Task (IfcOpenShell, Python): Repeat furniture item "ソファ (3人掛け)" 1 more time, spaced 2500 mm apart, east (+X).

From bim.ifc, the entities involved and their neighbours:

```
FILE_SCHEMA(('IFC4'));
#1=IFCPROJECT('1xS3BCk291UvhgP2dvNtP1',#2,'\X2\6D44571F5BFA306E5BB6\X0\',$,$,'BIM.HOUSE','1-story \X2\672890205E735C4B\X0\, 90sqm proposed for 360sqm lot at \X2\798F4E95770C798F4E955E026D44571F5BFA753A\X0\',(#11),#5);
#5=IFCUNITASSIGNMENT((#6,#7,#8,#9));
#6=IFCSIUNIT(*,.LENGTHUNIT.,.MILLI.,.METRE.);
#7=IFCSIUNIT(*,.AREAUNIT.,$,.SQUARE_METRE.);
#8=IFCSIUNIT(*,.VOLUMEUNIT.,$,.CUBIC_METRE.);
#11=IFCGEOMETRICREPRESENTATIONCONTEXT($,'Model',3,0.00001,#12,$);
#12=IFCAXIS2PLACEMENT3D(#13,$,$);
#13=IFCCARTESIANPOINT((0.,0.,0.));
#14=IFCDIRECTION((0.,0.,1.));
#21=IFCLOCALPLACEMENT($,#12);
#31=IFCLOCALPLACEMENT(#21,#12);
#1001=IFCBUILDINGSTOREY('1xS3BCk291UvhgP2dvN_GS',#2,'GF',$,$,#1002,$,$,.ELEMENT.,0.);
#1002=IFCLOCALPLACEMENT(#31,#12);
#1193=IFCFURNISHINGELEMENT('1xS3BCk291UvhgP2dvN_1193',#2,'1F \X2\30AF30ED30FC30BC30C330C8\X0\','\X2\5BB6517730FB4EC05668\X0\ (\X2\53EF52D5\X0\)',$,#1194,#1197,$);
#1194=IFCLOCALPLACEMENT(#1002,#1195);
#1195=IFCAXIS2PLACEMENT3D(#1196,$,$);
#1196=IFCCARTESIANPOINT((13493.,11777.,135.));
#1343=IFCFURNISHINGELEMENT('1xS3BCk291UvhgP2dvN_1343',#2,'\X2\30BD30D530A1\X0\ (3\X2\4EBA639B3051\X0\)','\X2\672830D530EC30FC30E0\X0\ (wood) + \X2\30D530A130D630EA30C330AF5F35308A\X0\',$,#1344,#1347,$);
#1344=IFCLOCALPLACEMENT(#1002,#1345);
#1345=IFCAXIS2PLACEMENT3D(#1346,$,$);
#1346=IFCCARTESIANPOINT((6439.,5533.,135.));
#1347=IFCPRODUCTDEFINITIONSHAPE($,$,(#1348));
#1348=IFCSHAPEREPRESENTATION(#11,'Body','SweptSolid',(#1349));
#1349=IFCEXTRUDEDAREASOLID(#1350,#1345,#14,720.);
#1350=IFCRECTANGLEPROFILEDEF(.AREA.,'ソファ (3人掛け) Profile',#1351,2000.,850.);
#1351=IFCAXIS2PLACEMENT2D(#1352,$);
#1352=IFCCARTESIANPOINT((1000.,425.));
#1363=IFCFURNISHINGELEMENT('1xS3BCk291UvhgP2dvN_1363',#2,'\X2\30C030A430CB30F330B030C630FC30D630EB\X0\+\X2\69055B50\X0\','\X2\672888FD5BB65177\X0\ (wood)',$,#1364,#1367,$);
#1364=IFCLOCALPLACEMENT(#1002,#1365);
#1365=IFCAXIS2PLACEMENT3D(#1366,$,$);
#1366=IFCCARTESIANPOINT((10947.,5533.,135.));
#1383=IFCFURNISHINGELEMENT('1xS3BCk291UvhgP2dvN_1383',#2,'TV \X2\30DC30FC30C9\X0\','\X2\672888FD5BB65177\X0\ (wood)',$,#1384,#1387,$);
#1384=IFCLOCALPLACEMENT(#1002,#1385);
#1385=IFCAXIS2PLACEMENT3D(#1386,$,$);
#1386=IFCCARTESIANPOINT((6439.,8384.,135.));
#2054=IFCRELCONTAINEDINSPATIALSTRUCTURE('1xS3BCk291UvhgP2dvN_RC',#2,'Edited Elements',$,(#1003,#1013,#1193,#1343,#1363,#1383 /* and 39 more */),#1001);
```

```python
import numpy as np
import ifcopenshell
import ifcopenshell.api.geometry
import ifcopenshell.api.root
import ifcopenshell.util.element
import ifcopenshell.util.placement
import ifcopenshell.util.unit

model = ifcopenshell.open("bim.ifc")
unit_scale = ifcopenshell.util.unit.calculate_unit_scale(model)


def reuse_history(source, copy):
    """copy_class also copies each property set's owner history, people and application; keep the originals."""
    for rel in copy.IsDefinedBy:
        if rel.is_a("IfcRelDefinesByProperties") and (history := rel.RelatingPropertyDefinition.OwnerHistory):
            rel.RelatingPropertyDefinition.OwnerHistory = source.OwnerHistory
            ifcopenshell.util.element.remove_deep2(model, history)


source = model.by_guid("1xS3BCk291UvhgP2dvN_1343")
base = ifcopenshell.util.placement.get_local_placement(source.ObjectPlacement)
step = np.array([1.0, 0.0, 0.0]) * 2.5 / unit_scale

for i in range(1, 2):
    copy = ifcopenshell.api.root.copy_class(model, product=source)
    copy.Representation = ifcopenshell.util.element.copy_deep(
        model, source.Representation, exclude=["IfcGeometricRepresentationContext", "IfcRepresentationMap"]
    )
    reuse_history(source, copy)
    matrix = base.copy()
    matrix[:3, 3] += i * step
    print("added at", matrix[:3, 3].round(3) + 0.0)
    ifcopenshell.api.geometry.edit_object_placement(model, product=copy, matrix=matrix, is_si=False)

model.write("bim_rev.ifc")
```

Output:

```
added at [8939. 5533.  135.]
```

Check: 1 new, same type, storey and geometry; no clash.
